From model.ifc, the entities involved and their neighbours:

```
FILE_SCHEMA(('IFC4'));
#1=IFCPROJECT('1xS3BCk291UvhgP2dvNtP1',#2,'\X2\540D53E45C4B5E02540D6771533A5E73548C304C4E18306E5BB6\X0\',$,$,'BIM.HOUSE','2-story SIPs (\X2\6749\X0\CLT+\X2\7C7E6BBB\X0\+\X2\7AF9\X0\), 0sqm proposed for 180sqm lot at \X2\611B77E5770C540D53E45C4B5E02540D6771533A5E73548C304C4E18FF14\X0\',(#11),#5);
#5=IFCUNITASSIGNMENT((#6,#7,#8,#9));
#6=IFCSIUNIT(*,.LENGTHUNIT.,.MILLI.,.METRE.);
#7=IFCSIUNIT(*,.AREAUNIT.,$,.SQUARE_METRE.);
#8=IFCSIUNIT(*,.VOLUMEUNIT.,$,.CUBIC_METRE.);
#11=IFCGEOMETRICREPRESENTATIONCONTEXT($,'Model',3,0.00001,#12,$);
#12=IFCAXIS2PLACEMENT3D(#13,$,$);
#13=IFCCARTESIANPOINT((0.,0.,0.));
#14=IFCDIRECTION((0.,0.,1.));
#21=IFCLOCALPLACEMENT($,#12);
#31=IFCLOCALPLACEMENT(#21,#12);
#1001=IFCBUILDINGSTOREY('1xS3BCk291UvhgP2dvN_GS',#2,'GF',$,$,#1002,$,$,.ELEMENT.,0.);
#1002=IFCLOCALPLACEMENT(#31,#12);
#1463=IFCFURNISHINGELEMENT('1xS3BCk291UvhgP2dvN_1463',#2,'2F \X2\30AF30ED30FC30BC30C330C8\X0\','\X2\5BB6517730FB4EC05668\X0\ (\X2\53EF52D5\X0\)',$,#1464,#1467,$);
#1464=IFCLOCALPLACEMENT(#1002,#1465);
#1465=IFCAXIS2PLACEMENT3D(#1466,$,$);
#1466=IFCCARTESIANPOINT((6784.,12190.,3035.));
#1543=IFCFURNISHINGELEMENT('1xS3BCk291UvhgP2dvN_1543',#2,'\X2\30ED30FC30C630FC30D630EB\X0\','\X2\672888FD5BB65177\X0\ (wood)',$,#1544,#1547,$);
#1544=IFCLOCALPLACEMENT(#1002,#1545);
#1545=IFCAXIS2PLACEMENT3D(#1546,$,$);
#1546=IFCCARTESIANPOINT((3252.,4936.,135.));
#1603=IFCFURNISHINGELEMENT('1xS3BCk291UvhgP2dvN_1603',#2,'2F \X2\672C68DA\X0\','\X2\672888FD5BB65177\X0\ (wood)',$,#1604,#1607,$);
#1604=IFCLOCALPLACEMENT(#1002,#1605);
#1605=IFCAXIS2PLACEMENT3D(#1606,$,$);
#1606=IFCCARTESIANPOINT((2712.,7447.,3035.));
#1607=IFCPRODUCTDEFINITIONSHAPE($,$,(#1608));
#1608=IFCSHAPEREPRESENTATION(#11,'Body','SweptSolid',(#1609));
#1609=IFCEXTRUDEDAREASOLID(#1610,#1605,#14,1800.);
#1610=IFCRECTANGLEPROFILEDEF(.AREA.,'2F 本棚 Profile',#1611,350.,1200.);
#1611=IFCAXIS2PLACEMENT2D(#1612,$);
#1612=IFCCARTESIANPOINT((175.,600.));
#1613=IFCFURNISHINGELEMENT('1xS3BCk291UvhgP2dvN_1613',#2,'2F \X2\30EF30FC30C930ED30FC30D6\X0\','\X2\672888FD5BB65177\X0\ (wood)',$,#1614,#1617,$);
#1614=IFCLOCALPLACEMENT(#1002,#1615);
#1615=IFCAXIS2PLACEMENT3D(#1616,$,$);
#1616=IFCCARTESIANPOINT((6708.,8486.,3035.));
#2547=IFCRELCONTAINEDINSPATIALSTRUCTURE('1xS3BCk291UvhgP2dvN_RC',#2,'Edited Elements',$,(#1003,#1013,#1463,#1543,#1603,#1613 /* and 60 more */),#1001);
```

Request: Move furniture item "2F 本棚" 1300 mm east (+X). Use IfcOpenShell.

```python
import ifcopenshell
import ifcopenshell.api.geometry
import ifcopenshell.util.placement

model = ifcopenshell.open("model.ifc")

item = model.by_id(1603)
matrix = ifcopenshell.util.placement.get_local_placement(item.ObjectPlacement)
matrix[0, 3] += 1300.0
ifcopenshell.api.geometry.edit_object_placement(model, product=item, matrix=matrix, is_si=False)

print(ifcopenshell.util.placement.get_local_placement(item.ObjectPlacement).round(3) + 0.0)

model.write("model_updated.ifc")
```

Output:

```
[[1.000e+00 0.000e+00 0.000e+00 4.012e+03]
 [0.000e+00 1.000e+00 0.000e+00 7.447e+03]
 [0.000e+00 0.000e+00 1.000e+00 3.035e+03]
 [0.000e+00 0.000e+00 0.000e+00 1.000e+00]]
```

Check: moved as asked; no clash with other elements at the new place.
